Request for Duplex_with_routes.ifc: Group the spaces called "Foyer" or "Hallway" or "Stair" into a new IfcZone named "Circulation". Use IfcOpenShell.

First a look at what the model holds.

```python
import ifcopenshell

model = ifcopenshell.open("Duplex_with_routes.ifc")
print(model.schema)
seen = {}
for space in model.by_type("IfcSpace"):
    seen[space.LongName] = seen.get(space.LongName, 0) + 1
for name, count in sorted(seen.items(), key=str):
    print(count, "x", name)
print("zones:", [z.Name for z in model.by_type("IfcZone")][:20])
```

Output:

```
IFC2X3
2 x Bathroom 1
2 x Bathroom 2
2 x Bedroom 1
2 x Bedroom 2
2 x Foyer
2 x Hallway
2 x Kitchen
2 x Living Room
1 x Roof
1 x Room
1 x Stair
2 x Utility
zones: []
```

```python
import ifcopenshell
import ifcopenshell.api.group
import ifcopenshell.api.root

model = ifcopenshell.open("Duplex_with_routes.ifc")

names = {"Foyer", "Hallway", "Stair"}
spaces = [s for s in model.by_type("IfcSpace") if s.LongName in names]

zone = ifcopenshell.api.root.create_entity(model, ifc_class="IfcZone", name="Circulation")
ifcopenshell.api.group.assign_group(model, products=spaces, group=zone)
print(len(spaces), "spaces in", zone.Name)

model.write("Duplex_with_routes_edited.ifc")
```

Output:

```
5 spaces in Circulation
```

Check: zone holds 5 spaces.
